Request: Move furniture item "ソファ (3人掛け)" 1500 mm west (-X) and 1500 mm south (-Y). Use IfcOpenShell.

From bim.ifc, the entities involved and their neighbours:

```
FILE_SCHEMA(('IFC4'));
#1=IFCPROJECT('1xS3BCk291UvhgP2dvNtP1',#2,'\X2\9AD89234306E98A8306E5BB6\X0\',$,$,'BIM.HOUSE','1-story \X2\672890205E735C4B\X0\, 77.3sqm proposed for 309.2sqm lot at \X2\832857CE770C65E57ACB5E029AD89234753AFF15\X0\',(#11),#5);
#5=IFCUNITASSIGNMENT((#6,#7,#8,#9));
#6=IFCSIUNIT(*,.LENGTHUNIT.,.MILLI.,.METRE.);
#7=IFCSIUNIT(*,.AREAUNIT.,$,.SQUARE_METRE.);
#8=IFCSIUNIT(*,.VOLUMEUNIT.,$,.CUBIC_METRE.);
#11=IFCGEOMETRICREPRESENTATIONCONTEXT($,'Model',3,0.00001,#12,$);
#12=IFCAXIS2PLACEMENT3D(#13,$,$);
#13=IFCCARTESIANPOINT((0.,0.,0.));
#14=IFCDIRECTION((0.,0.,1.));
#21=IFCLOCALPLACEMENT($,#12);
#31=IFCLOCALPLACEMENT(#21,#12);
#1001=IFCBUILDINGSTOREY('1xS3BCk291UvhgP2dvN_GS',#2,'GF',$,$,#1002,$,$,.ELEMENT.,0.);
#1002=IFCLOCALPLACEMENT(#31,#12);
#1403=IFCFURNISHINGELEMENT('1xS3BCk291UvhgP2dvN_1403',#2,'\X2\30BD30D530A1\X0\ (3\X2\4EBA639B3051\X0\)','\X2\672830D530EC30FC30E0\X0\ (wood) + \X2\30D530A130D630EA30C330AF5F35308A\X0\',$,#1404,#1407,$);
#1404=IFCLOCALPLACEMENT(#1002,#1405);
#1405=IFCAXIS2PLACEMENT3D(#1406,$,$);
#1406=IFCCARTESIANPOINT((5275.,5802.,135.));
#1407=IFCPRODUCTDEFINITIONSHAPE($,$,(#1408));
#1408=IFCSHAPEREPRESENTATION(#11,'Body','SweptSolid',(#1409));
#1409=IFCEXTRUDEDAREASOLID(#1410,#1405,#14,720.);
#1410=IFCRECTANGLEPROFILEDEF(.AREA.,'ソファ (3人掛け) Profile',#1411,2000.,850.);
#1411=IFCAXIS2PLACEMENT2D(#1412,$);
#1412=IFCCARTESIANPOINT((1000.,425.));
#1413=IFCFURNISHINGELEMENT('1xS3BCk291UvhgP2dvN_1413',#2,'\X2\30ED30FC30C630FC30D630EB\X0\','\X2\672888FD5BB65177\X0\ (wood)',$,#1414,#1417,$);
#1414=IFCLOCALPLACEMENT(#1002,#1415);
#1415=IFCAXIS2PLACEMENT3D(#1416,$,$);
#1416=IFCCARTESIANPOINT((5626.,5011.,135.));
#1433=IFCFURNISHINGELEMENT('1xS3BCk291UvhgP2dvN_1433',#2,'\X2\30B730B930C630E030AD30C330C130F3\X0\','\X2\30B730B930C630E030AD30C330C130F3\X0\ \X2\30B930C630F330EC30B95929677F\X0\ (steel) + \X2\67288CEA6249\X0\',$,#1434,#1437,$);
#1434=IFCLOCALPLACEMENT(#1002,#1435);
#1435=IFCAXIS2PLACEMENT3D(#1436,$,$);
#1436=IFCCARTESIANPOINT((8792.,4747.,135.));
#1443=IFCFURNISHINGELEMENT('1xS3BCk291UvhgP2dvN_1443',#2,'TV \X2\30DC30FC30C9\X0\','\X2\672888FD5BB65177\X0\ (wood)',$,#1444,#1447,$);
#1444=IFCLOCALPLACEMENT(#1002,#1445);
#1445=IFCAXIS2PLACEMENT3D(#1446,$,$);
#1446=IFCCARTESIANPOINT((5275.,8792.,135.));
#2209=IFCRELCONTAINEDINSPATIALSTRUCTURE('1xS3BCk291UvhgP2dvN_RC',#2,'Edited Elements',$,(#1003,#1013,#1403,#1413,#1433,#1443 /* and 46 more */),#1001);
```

```python
import ifcopenshell
import ifcopenshell.api.geometry
import ifcopenshell.util.placement

model = ifcopenshell.open("bim.ifc")

item = model.by_guid("1xS3BCk291UvhgP2dvN_1403")
matrix = ifcopenshell.util.placement.get_local_placement(item.ObjectPlacement)
matrix[0, 3] -= 1500.0
matrix[1, 3] -= 1500.0
ifcopenshell.api.geometry.edit_object_placement(model, product=item, matrix=matrix, is_si=False)

print(ifcopenshell.util.placement.get_local_placement(item.ObjectPlacement).round(3) + 0.0)

model.write("bim_updated.ifc")
```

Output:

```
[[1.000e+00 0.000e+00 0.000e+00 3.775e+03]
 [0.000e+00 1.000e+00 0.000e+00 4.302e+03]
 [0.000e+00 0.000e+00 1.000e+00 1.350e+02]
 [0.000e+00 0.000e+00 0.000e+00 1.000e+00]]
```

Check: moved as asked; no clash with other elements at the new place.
